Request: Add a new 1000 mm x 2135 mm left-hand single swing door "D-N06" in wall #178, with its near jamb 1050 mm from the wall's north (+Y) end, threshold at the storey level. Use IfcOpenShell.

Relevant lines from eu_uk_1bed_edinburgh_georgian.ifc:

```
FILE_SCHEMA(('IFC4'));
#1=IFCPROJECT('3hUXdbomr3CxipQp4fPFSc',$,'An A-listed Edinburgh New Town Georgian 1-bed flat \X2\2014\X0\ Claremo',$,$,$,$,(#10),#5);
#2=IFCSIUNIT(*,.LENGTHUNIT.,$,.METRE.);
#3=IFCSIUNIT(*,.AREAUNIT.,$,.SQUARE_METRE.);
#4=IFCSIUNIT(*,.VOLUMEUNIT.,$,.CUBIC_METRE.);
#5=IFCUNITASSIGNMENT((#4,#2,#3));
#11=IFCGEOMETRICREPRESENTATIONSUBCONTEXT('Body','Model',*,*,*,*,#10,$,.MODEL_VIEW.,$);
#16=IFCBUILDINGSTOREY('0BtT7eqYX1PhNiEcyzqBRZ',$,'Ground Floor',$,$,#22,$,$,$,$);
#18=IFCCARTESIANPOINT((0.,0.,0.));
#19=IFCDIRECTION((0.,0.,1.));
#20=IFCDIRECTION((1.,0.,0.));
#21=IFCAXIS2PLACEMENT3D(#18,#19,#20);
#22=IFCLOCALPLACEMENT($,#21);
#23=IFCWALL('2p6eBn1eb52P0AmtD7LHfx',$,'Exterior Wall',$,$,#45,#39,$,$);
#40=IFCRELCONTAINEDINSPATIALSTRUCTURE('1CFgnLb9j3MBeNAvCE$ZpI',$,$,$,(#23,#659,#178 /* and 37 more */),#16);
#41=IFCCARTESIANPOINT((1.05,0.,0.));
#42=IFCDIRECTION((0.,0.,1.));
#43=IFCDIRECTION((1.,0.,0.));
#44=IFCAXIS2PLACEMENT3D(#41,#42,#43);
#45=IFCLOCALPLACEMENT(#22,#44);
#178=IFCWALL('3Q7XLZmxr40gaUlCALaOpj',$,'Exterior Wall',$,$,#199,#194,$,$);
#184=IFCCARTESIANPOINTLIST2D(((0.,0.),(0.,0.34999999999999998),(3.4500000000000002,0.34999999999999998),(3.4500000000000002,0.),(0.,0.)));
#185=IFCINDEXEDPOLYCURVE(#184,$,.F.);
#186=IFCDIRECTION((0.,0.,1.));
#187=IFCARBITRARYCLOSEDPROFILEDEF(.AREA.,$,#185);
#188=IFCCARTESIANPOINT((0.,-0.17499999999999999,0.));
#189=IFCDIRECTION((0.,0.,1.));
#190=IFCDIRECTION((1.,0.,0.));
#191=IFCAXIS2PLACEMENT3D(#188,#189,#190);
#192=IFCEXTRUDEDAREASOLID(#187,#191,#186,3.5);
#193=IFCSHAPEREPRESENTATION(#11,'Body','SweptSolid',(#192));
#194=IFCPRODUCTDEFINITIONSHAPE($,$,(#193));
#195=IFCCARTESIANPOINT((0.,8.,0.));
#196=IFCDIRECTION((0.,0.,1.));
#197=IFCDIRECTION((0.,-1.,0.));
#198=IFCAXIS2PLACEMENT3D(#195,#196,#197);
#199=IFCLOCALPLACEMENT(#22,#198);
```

```python
import numpy as np
import ifcopenshell
import ifcopenshell.api.feature
import ifcopenshell.api.geometry
import ifcopenshell.api.root
import ifcopenshell.api.spatial
import ifcopenshell.geom
import ifcopenshell.util.element
import ifcopenshell.util.placement
import ifcopenshell.util.representation
import ifcopenshell.util.shape
import ifcopenshell.util.unit

model = ifcopenshell.open("eu_uk_1bed_edinburgh_georgian.ifc")
unit_scale = ifcopenshell.util.unit.calculate_unit_scale(model)
settings = ifcopenshell.geom.settings()


def volume(element):
    """Net volume in cubic metres, openings subtracted."""
    shape = ifcopenshell.geom.create_shape(settings, element)
    return ifcopenshell.util.shape.get_volume(shape.geometry)


wall = model.by_guid("3Q7XLZmxr40gaUlCALaOpj")
storey = ifcopenshell.util.element.get_container(wall, ifc_class="IfcBuildingStorey")
context = ifcopenshell.util.representation.get_context(model, "Model", "Body", "MODEL_VIEW")
before = volume(wall)

width, height, from_end, sill = 1, 2.135, 1.05, 0.0  # metres

# The wall runs along its own X axis, and the end named is its -X end.
wall_shape = ifcopenshell.geom.create_shape(settings, wall)
x, y, z = ifcopenshell.util.shape.get_vertices(wall_shape.geometry).T
start = x.min() + from_end
face, thickness = float(y.min()), float(y.max() - y.min())
wall_matrix = ifcopenshell.util.placement.get_local_placement(wall.ObjectPlacement)
level = ifcopenshell.util.placement.get_local_placement(storey.ObjectPlacement)[2, 3]


def in_wall(x, y):
    """Placement at x, y metres in the wall's axes, at sill height."""
    matrix = wall_matrix.copy()
    matrix[:, 3] = wall_matrix @ np.array([x / unit_scale, y / unit_scale, 0.0, 1.0])
    matrix[2, 3] = level + sill / unit_scale
    return matrix


# Opening: a box that overshoots both wall faces by 50 mm.
opening = ifcopenshell.api.root.create_entity(model, ifc_class="IfcOpeningElement", predefined_type="OPENING")
box = ifcopenshell.api.geometry.add_wall_representation(
    model, context=context, length=width, height=height, thickness=thickness + 0.1
)
ifcopenshell.api.geometry.assign_representation(model, product=opening, representation=box)
ifcopenshell.api.geometry.edit_object_placement(model, product=opening, matrix=in_wall(start, face - 0.05), is_si=False)
ifcopenshell.api.feature.add_feature(model, feature=opening, element=wall)

door = ifcopenshell.api.root.create_entity(model, ifc_class="IfcDoor", name="D-N06", predefined_type="DOOR")
door.OverallWidth, door.OverallHeight = width / unit_scale, height / unit_scale
door.OperationType = "SINGLE_SWING_LEFT"
body = ifcopenshell.api.geometry.add_door_representation(
    model,
    context=context,
    overall_width=door.OverallWidth,
    overall_height=door.OverallHeight,
    operation_type="SINGLE_SWING_LEFT",
    lining_properties={"LiningDepth": thickness / unit_scale, "ThresholdDepth": thickness / unit_scale},
)
ifcopenshell.api.geometry.assign_representation(model, product=door, representation=body)
ifcopenshell.api.spatial.assign_container(model, products=[door], relating_structure=storey)
ifcopenshell.api.feature.add_filling(model, opening=opening, element=door)

# The lining spans the wall, so the door starts at the wall face.
ifcopenshell.api.geometry.edit_object_placement(model, product=door, matrix=in_wall(start, face), is_si=False)

after = volume(wall)

print(f"wall volume {before:.3f} -> {after:.3f} m3")

model.write("eu_uk_1bed_edinburgh_georgian-out.ifc")
```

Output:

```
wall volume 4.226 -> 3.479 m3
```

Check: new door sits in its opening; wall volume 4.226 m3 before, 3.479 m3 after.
